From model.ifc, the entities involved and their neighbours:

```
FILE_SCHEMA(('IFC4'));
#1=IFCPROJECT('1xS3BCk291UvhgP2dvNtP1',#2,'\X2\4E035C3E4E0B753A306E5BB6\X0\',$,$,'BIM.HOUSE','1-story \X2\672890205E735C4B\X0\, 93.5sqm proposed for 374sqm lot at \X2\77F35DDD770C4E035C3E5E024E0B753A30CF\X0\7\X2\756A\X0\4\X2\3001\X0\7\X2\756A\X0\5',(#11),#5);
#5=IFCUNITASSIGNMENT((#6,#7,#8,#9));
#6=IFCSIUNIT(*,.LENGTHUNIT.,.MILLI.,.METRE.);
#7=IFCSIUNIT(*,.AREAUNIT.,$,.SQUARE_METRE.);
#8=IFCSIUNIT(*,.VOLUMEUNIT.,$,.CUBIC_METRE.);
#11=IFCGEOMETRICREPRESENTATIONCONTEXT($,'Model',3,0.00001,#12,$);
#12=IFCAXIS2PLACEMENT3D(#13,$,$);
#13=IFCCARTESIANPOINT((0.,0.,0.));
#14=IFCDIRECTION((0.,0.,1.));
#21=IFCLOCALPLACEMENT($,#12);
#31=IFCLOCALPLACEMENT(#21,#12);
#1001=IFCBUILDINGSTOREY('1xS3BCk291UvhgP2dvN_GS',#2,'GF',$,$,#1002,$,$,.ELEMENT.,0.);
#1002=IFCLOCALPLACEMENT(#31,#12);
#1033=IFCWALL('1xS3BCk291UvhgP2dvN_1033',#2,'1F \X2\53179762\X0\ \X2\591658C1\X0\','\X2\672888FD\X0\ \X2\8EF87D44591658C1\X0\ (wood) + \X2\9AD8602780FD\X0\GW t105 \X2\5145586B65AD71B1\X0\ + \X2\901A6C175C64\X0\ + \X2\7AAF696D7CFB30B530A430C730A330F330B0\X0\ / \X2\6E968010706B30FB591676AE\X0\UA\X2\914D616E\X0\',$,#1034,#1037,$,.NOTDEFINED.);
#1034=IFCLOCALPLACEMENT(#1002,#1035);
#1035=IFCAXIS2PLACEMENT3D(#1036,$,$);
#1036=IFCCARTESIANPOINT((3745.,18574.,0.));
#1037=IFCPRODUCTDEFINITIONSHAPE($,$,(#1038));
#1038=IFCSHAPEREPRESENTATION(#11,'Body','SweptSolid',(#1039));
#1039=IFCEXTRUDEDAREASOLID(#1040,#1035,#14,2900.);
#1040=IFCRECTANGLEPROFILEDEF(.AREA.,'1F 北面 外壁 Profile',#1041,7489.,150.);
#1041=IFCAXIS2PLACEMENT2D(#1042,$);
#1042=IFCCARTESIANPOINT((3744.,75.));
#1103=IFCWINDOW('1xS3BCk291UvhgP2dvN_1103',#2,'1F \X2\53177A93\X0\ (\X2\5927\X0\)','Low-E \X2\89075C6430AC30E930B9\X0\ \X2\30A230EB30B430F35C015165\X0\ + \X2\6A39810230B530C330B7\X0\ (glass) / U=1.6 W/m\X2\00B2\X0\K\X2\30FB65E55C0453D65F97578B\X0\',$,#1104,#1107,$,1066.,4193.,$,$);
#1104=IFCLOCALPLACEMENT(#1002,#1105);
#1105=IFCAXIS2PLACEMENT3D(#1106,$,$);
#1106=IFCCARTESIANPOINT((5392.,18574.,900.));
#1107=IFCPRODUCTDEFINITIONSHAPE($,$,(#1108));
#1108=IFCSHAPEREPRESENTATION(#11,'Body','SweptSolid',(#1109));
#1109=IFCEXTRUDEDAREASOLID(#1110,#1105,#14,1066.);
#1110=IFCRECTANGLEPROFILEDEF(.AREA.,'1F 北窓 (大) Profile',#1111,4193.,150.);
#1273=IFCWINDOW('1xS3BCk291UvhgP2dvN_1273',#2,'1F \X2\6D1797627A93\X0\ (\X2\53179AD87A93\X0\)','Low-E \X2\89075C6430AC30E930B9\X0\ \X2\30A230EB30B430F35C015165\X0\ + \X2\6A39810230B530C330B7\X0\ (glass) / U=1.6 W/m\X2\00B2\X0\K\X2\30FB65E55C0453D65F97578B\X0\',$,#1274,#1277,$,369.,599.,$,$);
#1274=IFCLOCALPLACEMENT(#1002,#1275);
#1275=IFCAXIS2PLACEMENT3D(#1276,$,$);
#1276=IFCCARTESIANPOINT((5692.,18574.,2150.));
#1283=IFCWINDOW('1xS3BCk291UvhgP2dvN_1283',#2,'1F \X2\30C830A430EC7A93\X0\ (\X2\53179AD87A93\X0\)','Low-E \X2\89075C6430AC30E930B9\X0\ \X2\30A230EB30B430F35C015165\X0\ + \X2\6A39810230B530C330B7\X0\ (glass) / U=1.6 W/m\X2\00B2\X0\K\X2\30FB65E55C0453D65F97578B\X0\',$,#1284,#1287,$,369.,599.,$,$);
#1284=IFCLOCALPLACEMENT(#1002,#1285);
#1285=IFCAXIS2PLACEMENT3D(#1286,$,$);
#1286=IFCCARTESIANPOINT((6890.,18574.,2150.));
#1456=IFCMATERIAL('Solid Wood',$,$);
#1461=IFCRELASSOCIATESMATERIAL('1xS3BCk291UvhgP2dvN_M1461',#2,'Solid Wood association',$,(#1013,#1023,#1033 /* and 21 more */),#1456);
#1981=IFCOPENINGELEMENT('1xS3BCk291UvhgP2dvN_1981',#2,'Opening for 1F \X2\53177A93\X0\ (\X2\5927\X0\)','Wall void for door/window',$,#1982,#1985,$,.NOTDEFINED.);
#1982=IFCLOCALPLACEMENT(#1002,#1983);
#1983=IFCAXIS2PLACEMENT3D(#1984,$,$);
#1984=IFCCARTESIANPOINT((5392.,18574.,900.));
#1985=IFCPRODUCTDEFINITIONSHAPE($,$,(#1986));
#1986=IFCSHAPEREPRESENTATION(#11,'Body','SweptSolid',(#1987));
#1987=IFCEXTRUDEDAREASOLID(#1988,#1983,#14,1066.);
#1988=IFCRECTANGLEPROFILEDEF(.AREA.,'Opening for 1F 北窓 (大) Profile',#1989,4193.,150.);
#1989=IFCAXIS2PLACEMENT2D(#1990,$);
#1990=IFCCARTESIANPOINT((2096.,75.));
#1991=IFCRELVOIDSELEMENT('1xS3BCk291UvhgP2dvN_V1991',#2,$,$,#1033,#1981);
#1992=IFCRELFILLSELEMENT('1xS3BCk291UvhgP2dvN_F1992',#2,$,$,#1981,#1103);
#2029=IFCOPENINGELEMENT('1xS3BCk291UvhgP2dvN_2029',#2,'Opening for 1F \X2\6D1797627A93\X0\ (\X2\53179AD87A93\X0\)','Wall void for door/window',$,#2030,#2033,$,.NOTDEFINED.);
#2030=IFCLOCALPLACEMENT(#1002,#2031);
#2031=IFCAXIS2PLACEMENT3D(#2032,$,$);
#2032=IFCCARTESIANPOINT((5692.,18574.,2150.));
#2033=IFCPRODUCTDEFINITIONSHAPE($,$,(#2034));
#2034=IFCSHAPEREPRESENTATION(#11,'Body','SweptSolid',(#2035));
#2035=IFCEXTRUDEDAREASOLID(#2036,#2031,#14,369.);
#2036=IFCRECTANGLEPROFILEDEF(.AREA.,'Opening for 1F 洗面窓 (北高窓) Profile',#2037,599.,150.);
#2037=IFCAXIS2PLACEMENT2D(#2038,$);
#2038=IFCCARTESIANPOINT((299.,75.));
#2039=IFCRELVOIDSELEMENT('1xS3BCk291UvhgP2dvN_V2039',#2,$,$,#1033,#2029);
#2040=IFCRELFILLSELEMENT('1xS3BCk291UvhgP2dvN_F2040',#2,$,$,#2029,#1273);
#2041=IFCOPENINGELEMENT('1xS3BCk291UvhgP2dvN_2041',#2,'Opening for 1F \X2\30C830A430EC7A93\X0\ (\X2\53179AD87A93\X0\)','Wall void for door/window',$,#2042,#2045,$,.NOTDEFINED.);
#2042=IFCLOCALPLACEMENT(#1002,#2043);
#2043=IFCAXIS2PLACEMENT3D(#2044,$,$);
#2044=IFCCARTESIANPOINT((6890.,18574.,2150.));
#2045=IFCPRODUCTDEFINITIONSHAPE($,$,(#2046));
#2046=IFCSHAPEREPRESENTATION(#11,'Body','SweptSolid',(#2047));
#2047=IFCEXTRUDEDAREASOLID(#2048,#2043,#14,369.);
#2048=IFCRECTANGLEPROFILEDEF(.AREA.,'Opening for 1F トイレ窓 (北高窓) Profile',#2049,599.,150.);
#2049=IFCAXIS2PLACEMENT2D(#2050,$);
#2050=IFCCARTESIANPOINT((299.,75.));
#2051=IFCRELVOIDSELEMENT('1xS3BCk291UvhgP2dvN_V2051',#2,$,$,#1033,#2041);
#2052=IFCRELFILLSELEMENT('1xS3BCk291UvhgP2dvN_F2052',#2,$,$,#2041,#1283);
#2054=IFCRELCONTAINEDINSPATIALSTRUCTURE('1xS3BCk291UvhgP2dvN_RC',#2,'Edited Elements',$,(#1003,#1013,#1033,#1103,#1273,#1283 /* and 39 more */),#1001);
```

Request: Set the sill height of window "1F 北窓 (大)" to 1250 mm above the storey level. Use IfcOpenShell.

```python
import numpy as np
import ifcopenshell
import ifcopenshell.api.geometry
import ifcopenshell.geom
import ifcopenshell.util.element
import ifcopenshell.util.placement
import ifcopenshell.util.shape
import ifcopenshell.util.unit

model = ifcopenshell.open("model.ifc")
unit_scale = ifcopenshell.util.unit.calculate_unit_scale(model)

window = model.by_guid("1xS3BCk291UvhgP2dvN_1103")
opening = window.FillsVoids[0].RelatingOpeningElement
storey = ifcopenshell.util.element.get_container(window, ifc_class="IfcBuildingStorey")
level = ifcopenshell.util.placement.get_local_placement(storey.ObjectPlacement)[2, 3]

# The opening's origin need not be at the sill, so measure its lowest point.
shape = ifcopenshell.geom.create_shape(ifcopenshell.geom.settings(), opening)
bottom = ifcopenshell.util.shape.get_shape_bottom_elevation(shape, shape.geometry) / unit_scale
dz = level + 1.25 / unit_scale - bottom

shift = np.array([0.0, 0.0, dz])
# The window is not placed relative to its opening, so move both.
for product in (opening, window):
    matrix = ifcopenshell.util.placement.get_local_placement(product.ObjectPlacement)
    matrix[:3, 3] += shift
    ifcopenshell.api.geometry.edit_object_placement(model, product=product, matrix=matrix, is_si=False)

print(f"moved by {dz * unit_scale:+.3f} m")

model.write("model_updated.ifc")
```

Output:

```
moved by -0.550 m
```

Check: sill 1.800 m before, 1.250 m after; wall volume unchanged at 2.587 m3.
